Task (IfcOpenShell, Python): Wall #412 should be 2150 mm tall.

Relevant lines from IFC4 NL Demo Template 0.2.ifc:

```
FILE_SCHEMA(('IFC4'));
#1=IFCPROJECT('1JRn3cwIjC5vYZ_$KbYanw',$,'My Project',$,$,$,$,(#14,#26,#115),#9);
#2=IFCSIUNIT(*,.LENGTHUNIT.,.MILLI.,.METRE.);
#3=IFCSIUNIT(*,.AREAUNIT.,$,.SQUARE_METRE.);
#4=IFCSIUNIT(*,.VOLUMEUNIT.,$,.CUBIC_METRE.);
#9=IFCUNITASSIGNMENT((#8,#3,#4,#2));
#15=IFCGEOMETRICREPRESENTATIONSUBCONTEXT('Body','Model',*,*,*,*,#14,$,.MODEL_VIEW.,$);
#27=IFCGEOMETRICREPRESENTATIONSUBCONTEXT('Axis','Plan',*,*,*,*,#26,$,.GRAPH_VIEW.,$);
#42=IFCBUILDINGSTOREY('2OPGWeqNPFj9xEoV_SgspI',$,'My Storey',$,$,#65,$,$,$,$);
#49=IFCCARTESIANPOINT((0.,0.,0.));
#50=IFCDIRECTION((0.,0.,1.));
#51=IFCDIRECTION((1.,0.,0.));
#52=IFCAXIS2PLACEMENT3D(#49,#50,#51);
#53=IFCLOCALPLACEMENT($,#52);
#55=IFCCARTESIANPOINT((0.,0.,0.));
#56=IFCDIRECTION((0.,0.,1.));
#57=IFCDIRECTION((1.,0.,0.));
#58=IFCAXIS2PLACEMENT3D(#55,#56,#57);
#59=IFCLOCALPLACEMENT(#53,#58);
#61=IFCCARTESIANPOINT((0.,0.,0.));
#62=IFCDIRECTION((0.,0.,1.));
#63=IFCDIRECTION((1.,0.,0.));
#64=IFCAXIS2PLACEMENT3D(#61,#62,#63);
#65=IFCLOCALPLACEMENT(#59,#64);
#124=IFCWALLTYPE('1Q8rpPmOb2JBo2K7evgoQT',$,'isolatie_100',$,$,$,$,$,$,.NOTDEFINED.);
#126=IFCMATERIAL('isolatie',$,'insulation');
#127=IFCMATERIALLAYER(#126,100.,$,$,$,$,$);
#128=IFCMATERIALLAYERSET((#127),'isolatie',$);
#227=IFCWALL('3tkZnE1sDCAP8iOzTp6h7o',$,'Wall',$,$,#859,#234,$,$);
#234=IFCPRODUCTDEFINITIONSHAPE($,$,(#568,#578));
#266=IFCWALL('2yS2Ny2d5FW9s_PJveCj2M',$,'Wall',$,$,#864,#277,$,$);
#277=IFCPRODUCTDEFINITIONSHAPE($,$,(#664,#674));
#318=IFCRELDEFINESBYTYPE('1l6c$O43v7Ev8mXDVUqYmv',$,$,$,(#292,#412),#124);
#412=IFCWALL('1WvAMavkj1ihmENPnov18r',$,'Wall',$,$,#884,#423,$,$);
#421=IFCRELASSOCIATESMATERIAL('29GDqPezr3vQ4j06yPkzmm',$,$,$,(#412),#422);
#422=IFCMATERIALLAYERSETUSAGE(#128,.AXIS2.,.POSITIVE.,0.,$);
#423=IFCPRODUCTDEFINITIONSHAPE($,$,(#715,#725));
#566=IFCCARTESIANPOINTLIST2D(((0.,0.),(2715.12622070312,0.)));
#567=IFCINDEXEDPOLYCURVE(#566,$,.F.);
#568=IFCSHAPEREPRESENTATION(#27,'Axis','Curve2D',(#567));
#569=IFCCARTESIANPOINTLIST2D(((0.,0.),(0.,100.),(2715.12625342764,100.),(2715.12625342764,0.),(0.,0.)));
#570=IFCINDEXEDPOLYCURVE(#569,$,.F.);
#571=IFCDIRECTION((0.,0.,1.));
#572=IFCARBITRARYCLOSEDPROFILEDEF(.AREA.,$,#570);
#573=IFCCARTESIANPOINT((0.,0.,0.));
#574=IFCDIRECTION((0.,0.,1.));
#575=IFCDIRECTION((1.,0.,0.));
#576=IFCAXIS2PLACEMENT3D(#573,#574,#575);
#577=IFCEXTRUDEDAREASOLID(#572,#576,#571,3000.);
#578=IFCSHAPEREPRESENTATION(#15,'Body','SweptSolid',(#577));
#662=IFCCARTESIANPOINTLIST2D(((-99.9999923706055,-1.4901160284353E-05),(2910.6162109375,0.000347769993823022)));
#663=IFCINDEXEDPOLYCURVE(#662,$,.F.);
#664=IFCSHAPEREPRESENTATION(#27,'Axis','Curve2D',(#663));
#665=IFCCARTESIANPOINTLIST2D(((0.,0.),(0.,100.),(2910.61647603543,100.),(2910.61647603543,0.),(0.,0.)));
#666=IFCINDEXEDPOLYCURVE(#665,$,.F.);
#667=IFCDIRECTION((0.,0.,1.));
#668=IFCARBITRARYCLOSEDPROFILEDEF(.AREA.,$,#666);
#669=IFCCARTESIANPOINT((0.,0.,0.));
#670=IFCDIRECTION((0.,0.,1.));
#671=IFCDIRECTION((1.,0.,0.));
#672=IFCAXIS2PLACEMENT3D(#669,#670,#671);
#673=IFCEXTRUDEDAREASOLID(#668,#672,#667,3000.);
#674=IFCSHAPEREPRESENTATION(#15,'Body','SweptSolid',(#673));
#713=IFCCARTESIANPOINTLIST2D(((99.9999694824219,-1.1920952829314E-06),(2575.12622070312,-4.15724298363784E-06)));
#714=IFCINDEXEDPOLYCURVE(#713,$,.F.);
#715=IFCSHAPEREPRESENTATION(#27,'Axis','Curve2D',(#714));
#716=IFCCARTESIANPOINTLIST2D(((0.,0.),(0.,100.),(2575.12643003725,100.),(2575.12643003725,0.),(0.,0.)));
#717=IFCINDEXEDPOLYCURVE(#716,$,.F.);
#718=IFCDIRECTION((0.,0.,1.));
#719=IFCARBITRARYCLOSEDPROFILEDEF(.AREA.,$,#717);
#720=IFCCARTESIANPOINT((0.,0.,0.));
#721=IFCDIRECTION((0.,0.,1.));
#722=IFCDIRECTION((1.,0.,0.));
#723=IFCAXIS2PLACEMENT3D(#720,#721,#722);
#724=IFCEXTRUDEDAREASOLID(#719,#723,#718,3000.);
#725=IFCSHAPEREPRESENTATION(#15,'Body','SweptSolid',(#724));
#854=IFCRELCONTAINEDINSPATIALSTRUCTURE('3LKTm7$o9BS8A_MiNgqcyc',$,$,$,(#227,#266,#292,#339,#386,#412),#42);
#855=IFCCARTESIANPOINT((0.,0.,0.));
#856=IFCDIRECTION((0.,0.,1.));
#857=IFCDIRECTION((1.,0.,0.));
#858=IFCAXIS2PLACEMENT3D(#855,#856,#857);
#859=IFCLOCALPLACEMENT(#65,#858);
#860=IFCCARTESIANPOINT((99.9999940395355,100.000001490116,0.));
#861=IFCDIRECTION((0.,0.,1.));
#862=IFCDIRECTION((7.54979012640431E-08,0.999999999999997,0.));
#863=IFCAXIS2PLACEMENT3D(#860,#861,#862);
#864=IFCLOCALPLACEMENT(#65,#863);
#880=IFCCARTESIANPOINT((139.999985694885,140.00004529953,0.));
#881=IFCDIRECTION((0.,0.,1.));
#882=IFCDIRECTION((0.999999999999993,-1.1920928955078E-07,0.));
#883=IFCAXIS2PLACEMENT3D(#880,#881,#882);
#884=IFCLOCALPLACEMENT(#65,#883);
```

```python
import ifcopenshell
import ifcopenshell.geom
import ifcopenshell.util.representation
import ifcopenshell.util.shape
import ifcopenshell.util.unit

model = ifcopenshell.open("IFC4 NL Demo Template 0.2.ifc")
unit_scale = ifcopenshell.util.unit.calculate_unit_scale(model)
settings = ifcopenshell.geom.settings()


def volume(element):
    """Net volume in cubic metres, openings subtracted."""
    shape = ifcopenshell.geom.create_shape(settings, element)
    return ifcopenshell.util.shape.get_volume(shape.geometry)


wall = model.by_guid("1WvAMavkj1ihmENPnov18r")
before = volume(wall)

body = ifcopenshell.util.representation.get_representation(wall, "Model", "Body")
solid = body.Items[0]
old_height = solid.Depth
solid.Depth = 2.15 / unit_scale
after = volume(wall)

print(f"height {old_height:g} -> {solid.Depth:g}, volume {before:.3f} -> {after:.3f} m3")

model.write("IFC4 NL Demo Template 0.2_edited.ifc")
```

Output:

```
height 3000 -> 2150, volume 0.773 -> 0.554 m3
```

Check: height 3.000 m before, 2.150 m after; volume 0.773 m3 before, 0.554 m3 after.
